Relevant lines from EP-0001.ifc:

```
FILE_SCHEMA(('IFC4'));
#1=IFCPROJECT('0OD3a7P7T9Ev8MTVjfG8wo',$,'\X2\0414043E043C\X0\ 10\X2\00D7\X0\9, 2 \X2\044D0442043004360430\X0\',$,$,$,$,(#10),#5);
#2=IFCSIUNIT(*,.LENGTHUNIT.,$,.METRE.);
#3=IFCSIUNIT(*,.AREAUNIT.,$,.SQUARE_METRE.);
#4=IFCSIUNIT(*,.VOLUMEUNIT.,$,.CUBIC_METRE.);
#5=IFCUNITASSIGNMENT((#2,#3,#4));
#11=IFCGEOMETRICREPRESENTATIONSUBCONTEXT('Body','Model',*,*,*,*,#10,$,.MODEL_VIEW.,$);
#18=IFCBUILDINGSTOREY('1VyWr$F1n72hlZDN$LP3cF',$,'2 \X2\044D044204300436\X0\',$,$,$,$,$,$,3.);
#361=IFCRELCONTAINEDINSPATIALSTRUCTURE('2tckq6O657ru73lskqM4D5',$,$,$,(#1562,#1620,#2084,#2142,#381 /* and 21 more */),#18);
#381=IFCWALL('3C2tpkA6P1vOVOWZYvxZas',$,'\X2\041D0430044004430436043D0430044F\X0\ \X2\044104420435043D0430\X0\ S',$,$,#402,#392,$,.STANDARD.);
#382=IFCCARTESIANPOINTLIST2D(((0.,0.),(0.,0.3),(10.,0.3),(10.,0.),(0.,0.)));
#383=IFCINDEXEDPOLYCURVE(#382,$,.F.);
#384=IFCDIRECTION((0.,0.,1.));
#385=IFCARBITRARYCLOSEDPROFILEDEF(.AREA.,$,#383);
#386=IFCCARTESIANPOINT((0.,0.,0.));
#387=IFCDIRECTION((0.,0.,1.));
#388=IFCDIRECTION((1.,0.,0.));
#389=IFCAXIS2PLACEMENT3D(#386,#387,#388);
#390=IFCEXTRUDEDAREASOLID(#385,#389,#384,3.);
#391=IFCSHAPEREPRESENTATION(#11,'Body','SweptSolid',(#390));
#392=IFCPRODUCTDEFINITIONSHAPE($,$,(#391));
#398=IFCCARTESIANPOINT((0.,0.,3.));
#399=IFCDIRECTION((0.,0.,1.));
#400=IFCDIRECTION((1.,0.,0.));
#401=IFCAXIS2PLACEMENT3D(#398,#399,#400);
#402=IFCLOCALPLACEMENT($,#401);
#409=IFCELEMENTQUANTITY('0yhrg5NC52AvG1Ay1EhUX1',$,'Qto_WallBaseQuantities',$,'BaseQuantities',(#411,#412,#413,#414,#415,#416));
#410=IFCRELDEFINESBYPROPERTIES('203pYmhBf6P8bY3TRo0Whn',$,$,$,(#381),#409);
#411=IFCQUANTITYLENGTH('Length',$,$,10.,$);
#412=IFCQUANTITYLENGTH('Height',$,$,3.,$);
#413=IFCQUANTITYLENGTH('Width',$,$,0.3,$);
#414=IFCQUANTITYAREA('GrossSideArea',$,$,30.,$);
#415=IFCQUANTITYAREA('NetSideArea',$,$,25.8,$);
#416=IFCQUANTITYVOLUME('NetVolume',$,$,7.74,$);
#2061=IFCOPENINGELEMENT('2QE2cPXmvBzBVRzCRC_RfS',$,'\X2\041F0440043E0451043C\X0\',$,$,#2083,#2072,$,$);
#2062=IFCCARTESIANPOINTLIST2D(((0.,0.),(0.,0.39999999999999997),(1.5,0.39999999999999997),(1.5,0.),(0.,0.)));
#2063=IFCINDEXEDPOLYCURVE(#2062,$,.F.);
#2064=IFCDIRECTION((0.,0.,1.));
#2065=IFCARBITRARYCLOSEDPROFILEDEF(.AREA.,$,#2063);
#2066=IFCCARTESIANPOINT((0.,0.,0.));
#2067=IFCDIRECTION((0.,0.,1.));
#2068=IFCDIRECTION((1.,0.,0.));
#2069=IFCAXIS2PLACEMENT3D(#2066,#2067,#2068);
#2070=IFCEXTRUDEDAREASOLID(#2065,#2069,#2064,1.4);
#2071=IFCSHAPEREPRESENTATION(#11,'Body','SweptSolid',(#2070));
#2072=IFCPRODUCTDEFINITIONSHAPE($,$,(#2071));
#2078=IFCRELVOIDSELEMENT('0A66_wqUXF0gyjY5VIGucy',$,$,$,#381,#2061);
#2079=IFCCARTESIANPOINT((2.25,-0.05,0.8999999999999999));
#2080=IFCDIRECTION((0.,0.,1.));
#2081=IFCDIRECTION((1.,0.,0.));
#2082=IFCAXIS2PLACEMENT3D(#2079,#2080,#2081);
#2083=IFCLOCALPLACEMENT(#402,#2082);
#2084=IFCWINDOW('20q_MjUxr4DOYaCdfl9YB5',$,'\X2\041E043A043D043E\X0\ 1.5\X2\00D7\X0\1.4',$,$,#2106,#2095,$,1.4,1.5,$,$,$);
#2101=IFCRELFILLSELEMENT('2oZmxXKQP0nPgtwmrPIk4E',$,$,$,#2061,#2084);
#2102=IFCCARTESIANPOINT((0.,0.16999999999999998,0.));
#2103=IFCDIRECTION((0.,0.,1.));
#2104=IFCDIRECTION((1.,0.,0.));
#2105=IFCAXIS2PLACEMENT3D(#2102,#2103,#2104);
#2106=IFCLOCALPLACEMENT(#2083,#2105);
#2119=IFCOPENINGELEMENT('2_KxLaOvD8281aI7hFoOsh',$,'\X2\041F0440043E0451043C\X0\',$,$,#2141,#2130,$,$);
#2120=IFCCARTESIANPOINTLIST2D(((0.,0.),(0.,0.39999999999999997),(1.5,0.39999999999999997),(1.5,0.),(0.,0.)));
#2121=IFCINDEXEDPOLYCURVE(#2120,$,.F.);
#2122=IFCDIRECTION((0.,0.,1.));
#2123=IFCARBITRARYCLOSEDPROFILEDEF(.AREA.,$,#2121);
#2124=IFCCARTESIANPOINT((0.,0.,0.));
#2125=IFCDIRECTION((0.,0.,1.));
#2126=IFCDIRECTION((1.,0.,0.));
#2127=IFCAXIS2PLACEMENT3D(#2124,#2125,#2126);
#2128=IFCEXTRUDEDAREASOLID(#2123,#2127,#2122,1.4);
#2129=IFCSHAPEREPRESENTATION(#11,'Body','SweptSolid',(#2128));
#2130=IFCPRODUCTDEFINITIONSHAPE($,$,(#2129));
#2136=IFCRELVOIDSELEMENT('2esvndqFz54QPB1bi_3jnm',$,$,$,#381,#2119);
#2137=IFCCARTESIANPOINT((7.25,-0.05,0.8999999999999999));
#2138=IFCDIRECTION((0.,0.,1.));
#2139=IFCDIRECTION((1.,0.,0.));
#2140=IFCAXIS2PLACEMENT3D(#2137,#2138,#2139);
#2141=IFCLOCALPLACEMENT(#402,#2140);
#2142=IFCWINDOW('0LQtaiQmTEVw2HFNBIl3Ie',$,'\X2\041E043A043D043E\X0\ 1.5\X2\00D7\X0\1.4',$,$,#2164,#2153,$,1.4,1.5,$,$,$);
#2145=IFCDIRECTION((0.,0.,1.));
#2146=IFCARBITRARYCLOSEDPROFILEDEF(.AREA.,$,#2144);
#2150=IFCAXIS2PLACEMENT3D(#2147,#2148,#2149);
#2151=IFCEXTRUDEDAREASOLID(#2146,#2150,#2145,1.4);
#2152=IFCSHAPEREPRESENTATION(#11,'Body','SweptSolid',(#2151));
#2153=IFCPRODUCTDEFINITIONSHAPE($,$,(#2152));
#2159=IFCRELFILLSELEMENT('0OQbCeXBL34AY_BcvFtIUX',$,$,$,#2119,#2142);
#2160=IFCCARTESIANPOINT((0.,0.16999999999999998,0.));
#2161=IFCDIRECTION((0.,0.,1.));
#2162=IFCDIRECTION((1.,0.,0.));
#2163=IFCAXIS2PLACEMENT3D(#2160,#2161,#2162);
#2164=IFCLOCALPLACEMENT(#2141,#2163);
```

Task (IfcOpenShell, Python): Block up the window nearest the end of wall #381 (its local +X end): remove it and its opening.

```python
import ifcopenshell
import ifcopenshell.api.feature
import ifcopenshell.api.pset
import ifcopenshell.api.root
import ifcopenshell.geom
import ifcopenshell.util.element
import ifcopenshell.util.shape
import ifcopenshell.util.unit

model = ifcopenshell.open("EP-0001.ifc")
area_scale = ifcopenshell.util.unit.calculate_unit_scale(model, "AREAUNIT")
volume_scale = ifcopenshell.util.unit.calculate_unit_scale(model, "VOLUMEUNIT")
settings = ifcopenshell.geom.settings()


def volume(element):
    """Net volume in cubic metres, openings subtracted."""
    shape = ifcopenshell.geom.create_shape(settings, element)
    return ifcopenshell.util.shape.get_volume(shape.geometry)


window = model.by_guid("0LQtaiQmTEVw2HFNBIl3Ie")
opening = window.FillsVoids[0].RelatingOpeningElement
wall = opening.VoidsElements[0].RelatingBuildingElement
before = volume(wall)

ifcopenshell.api.root.remove_product(model, product=window)
ifcopenshell.api.feature.remove_feature(model, feature=opening)

after = volume(wall)
thickness = 0.3  # wall thickness in metres

# Update the wall's stored quantities.
qto = model.by_id(ifcopenshell.util.element.get_pset(wall, "Qto_WallBaseQuantities", should_inherit=False)["id"])
ifcopenshell.api.pset.edit_qto(model, qto=qto, properties={
    "NetSideArea": after / thickness / area_scale,
    "NetVolume": after / volume_scale,
})

print(f"wall volume {before:.3f} -> {after:.3f} m3")

model.write("EP-0001_edited.ifc")
```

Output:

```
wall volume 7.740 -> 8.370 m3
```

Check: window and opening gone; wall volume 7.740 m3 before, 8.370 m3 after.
